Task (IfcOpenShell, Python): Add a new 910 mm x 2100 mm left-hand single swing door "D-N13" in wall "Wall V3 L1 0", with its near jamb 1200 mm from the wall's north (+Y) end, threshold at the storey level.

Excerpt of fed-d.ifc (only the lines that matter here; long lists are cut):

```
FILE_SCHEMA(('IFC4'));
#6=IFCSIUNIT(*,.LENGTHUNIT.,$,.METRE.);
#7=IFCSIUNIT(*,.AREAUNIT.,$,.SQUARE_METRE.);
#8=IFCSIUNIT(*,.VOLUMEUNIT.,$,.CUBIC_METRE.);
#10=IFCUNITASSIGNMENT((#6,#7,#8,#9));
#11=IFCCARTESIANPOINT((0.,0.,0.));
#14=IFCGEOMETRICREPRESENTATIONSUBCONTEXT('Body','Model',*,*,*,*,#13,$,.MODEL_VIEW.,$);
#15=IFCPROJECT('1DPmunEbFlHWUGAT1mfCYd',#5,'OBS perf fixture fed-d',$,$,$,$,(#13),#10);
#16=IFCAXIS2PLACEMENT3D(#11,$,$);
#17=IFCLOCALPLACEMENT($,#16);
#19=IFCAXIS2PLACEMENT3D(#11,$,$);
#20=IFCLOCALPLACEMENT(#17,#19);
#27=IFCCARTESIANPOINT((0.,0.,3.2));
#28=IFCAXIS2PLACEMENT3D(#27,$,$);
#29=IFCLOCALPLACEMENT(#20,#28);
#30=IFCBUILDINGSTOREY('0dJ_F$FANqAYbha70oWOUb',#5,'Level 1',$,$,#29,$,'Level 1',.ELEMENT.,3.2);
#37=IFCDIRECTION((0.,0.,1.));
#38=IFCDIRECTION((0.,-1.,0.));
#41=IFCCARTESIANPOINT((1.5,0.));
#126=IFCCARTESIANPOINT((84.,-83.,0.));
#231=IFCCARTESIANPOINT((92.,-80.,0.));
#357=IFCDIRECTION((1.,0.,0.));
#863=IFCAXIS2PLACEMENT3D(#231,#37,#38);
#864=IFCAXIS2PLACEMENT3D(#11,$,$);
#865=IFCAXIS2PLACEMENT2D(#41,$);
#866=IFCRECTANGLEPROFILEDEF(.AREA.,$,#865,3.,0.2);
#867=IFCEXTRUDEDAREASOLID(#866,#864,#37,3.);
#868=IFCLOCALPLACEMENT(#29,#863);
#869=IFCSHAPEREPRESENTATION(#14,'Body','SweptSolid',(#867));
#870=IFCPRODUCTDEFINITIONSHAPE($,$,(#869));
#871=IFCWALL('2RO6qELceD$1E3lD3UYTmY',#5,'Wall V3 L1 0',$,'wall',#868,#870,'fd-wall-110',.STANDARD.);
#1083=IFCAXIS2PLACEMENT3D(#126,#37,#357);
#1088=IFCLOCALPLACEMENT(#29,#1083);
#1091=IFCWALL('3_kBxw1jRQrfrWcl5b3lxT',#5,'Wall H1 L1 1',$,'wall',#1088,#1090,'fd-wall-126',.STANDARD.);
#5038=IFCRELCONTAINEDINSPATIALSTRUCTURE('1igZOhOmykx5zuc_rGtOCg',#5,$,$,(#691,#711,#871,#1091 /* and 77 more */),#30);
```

```python
import numpy as np
import ifcopenshell
import ifcopenshell.api.feature
import ifcopenshell.api.geometry
import ifcopenshell.api.root
import ifcopenshell.api.spatial
import ifcopenshell.geom
import ifcopenshell.util.element
import ifcopenshell.util.placement
import ifcopenshell.util.representation
import ifcopenshell.util.shape
import ifcopenshell.util.unit

model = ifcopenshell.open("fed-d.ifc")
unit_scale = ifcopenshell.util.unit.calculate_unit_scale(model)
settings = ifcopenshell.geom.settings()


def volume(element):
    """Net volume in cubic metres, openings subtracted."""
    shape = ifcopenshell.geom.create_shape(settings, element)
    return ifcopenshell.util.shape.get_volume(shape.geometry)


wall = model.by_guid("2RO6qELceD$1E3lD3UYTmY")
storey = ifcopenshell.util.element.get_container(wall, ifc_class="IfcBuildingStorey")
context = ifcopenshell.util.representation.get_context(model, "Model", "Body", "MODEL_VIEW")
before = volume(wall)

width, height, from_end, sill = 0.91, 2.1, 1.2, 0.0  # metres

# The wall runs along its own X axis, and the end named is its -X end.
wall_shape = ifcopenshell.geom.create_shape(settings, wall)
x, y, z = ifcopenshell.util.shape.get_vertices(wall_shape.geometry).T
start = x.min() + from_end
face, thickness = float(y.min()), float(y.max() - y.min())
wall_matrix = ifcopenshell.util.placement.get_local_placement(wall.ObjectPlacement)
level = ifcopenshell.util.placement.get_local_placement(storey.ObjectPlacement)[2, 3]


def in_wall(x, y):
    """Placement at x, y metres in the wall's axes, at sill height."""
    matrix = wall_matrix.copy()
    matrix[:, 3] = wall_matrix @ np.array([x / unit_scale, y / unit_scale, 0.0, 1.0])
    matrix[2, 3] = level + sill / unit_scale
    return matrix


# Opening: a box that overshoots both wall faces by 50 mm.
opening = ifcopenshell.api.root.create_entity(model, ifc_class="IfcOpeningElement", predefined_type="OPENING")
box = ifcopenshell.api.geometry.add_wall_representation(
    model, context=context, length=width, height=height, thickness=thickness + 0.1
)
ifcopenshell.api.geometry.assign_representation(model, product=opening, representation=box)
ifcopenshell.api.geometry.edit_object_placement(model, product=opening, matrix=in_wall(start, face - 0.05), is_si=False)
ifcopenshell.api.feature.add_feature(model, feature=opening, element=wall)

door = ifcopenshell.api.root.create_entity(model, ifc_class="IfcDoor", name="D-N13", predefined_type="DOOR")
door.OverallWidth, door.OverallHeight = width / unit_scale, height / unit_scale
door.OperationType = "SINGLE_SWING_LEFT"
body = ifcopenshell.api.geometry.add_door_representation(
    model,
    context=context,
    overall_width=door.OverallWidth,
    overall_height=door.OverallHeight,
    operation_type="SINGLE_SWING_LEFT",
    lining_properties={"LiningDepth": thickness / unit_scale, "ThresholdDepth": thickness / unit_scale},
)
ifcopenshell.api.geometry.assign_representation(model, product=door, representation=body)
ifcopenshell.api.spatial.assign_container(model, products=[door], relating_structure=storey)
ifcopenshell.api.feature.add_filling(model, opening=opening, element=door)

# The lining spans the wall, so the door starts at the wall face.
ifcopenshell.api.geometry.edit_object_placement(model, product=door, matrix=in_wall(start, face), is_si=False)

after = volume(wall)

print(f"wall volume {before:.3f} -> {after:.3f} m3")

model.write("fed-d_rev.ifc")
```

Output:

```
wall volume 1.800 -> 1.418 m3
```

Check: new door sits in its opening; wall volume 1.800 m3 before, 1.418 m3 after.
